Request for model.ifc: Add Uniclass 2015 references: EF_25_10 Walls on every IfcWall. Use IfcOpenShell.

First a look at what the model holds.

```python
import ifcopenshell

model = ifcopenshell.open("model.ifc")
print(model.schema)
print("classifications:", [c.Name for c in model.by_type("IfcClassification")])
for ifc_class in ("IfcDoor", "IfcRoof", "IfcStair", "IfcWall", "IfcWindow"):
    print(ifc_class, len(model.by_type(ifc_class)))
```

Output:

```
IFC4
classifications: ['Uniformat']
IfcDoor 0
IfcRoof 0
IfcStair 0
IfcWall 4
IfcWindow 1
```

```python
import ifcopenshell
import ifcopenshell.api.classification

model = ifcopenshell.open("model.ifc")

system = ifcopenshell.api.classification.add_classification(model, classification="Uniclass 2015")

codes = {
    "IfcWall": ("EF_25_10", "Walls"),
}
for ifc_class, (code, name) in codes.items():
    products = model.by_type(ifc_class)
    ifcopenshell.api.classification.add_reference(
        model, products=products, classification=system, identification=code, name=name
    )
    print(code, len(products))

model.write("model-out.ifc")
```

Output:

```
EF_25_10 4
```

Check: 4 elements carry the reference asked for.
